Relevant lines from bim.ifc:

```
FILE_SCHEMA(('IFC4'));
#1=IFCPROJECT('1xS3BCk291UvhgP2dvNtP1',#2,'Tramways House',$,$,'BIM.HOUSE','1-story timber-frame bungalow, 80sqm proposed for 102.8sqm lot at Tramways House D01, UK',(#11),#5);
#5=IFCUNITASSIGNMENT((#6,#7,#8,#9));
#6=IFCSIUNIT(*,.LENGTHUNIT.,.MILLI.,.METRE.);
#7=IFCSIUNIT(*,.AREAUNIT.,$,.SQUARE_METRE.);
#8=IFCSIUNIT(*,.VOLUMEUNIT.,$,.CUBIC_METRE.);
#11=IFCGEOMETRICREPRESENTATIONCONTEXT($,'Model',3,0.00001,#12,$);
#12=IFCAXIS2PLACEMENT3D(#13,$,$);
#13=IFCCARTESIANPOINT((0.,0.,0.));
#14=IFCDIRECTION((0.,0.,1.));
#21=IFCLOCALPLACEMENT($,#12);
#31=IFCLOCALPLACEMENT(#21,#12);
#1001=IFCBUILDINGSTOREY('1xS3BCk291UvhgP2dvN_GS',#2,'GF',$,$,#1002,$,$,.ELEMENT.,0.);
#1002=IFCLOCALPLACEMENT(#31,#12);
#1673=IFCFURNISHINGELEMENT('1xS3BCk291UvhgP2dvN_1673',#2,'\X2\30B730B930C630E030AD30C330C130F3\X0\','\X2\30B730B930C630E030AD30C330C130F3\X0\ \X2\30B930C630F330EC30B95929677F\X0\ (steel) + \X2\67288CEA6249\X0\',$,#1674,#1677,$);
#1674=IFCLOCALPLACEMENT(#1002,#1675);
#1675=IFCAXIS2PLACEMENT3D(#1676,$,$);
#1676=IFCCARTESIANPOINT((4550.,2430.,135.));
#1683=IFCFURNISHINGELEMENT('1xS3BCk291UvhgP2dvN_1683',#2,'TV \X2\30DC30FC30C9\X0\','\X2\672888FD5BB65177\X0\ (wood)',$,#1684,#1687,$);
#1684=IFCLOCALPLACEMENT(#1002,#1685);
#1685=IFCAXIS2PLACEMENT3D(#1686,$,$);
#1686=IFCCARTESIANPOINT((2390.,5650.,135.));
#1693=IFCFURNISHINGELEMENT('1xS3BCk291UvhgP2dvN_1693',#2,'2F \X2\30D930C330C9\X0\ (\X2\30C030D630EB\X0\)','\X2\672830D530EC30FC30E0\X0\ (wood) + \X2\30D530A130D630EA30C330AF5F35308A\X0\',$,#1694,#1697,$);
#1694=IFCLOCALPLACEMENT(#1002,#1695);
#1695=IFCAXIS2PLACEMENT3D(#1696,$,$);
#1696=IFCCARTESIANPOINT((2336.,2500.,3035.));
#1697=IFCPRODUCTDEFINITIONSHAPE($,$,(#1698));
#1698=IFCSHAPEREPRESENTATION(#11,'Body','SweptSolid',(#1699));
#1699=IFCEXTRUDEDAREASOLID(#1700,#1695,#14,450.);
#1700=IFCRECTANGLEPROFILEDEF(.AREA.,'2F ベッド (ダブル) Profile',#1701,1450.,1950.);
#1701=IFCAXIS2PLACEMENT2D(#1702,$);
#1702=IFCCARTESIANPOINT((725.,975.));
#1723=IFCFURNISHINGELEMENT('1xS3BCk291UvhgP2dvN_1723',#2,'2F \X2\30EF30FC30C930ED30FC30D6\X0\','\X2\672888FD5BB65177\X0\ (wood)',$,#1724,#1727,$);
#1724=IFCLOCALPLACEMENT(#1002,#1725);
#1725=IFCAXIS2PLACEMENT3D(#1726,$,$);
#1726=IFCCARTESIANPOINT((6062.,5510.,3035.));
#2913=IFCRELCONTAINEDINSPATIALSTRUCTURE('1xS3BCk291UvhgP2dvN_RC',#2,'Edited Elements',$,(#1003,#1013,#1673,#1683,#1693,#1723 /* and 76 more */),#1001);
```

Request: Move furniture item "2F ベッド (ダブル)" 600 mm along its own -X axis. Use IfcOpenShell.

```python
import ifcopenshell
import ifcopenshell.api.geometry
import ifcopenshell.util.placement

model = ifcopenshell.open("bim.ifc")

item = model.by_id(1693)
matrix = ifcopenshell.util.placement.get_local_placement(item.ObjectPlacement)
matrix[:3, 3] -= matrix[:3, 0] * 600.0
ifcopenshell.api.geometry.edit_object_placement(model, product=item, matrix=matrix, is_si=False)

print(ifcopenshell.util.placement.get_local_placement(item.ObjectPlacement).round(3) + 0.0)

model.write("bim-out.ifc")
```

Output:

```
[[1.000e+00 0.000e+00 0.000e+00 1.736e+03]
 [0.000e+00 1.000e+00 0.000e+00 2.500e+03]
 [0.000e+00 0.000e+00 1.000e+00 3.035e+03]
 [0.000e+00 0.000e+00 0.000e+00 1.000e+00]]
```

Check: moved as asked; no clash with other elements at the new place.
